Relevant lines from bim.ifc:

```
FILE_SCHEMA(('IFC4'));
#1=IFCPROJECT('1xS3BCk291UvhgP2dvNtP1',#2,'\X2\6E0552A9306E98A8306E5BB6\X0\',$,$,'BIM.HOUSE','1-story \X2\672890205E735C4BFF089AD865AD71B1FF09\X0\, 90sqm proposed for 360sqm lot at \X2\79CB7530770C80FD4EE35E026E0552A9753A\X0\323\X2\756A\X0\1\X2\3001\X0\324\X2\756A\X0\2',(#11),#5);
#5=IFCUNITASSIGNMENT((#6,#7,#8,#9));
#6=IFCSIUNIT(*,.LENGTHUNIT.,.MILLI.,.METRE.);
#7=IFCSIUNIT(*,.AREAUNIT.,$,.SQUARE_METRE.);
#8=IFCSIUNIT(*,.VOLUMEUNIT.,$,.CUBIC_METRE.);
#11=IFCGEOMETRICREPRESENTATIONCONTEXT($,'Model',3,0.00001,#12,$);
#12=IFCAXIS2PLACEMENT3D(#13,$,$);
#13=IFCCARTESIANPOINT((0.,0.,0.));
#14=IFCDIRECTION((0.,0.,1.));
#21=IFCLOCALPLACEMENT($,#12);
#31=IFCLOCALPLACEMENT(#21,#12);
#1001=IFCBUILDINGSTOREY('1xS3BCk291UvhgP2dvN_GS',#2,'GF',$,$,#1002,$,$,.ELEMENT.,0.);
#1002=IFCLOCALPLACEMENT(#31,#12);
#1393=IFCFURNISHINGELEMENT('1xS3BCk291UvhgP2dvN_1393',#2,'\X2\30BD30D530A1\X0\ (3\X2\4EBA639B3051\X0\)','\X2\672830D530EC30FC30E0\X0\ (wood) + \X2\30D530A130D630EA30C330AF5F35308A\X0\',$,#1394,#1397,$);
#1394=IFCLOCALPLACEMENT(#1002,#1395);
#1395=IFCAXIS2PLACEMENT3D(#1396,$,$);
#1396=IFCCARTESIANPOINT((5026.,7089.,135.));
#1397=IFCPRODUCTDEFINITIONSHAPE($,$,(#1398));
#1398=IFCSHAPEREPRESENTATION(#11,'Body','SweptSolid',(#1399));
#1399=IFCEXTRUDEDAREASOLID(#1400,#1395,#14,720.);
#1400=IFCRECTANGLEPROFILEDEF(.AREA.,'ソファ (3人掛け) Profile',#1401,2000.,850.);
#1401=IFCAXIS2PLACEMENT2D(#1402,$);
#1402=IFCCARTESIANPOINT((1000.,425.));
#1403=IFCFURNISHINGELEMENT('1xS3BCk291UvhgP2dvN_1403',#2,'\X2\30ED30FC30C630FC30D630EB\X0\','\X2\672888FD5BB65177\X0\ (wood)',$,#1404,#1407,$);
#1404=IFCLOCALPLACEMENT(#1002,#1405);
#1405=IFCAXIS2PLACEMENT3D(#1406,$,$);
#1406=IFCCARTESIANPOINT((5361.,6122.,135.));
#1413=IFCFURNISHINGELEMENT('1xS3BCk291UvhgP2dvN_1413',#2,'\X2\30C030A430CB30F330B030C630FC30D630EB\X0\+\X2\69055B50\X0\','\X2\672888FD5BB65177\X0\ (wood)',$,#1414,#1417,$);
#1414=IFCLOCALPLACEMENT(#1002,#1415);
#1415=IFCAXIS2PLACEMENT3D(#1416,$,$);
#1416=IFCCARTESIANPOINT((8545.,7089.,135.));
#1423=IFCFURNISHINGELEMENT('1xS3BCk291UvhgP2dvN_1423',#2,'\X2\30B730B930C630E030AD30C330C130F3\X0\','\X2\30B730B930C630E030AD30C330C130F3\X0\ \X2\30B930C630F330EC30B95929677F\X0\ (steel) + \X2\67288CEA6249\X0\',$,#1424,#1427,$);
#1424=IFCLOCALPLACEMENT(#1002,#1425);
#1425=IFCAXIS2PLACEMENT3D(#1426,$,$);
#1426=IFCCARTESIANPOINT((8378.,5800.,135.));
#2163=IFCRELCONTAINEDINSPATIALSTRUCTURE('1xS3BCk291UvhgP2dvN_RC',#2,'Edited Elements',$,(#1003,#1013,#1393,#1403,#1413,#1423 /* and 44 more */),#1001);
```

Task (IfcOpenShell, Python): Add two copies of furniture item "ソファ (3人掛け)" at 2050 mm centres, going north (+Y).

```python
import numpy as np
import ifcopenshell
import ifcopenshell.api.geometry
import ifcopenshell.api.root
import ifcopenshell.util.element
import ifcopenshell.util.placement
import ifcopenshell.util.unit

model = ifcopenshell.open("bim.ifc")
unit_scale = ifcopenshell.util.unit.calculate_unit_scale(model)


def reuse_history(source, copy):
    """copy_class also copies each property set's owner history, people and application; keep the originals."""
    for rel in copy.IsDefinedBy:
        if rel.is_a("IfcRelDefinesByProperties") and (history := rel.RelatingPropertyDefinition.OwnerHistory):
            rel.RelatingPropertyDefinition.OwnerHistory = source.OwnerHistory
            ifcopenshell.util.element.remove_deep2(model, history)


source = model.by_guid("1xS3BCk291UvhgP2dvN_1393")
base = ifcopenshell.util.placement.get_local_placement(source.ObjectPlacement)
step = np.array([0.0, 1.0, 0.0]) * 2.05 / unit_scale

for i in range(1, 3):
    copy = ifcopenshell.api.root.copy_class(model, product=source)
    copy.Representation = ifcopenshell.util.element.copy_deep(
        model, source.Representation, exclude=["IfcGeometricRepresentationContext", "IfcRepresentationMap"]
    )
    reuse_history(source, copy)
    matrix = base.copy()
    matrix[:3, 3] += i * step
    print("added at", matrix[:3, 3].round(3) + 0.0)
    ifcopenshell.api.geometry.edit_object_placement(model, product=copy, matrix=matrix, is_si=False)

model.write("bim-out.ifc")
```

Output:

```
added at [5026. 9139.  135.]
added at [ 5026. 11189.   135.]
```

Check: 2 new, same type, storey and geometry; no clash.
